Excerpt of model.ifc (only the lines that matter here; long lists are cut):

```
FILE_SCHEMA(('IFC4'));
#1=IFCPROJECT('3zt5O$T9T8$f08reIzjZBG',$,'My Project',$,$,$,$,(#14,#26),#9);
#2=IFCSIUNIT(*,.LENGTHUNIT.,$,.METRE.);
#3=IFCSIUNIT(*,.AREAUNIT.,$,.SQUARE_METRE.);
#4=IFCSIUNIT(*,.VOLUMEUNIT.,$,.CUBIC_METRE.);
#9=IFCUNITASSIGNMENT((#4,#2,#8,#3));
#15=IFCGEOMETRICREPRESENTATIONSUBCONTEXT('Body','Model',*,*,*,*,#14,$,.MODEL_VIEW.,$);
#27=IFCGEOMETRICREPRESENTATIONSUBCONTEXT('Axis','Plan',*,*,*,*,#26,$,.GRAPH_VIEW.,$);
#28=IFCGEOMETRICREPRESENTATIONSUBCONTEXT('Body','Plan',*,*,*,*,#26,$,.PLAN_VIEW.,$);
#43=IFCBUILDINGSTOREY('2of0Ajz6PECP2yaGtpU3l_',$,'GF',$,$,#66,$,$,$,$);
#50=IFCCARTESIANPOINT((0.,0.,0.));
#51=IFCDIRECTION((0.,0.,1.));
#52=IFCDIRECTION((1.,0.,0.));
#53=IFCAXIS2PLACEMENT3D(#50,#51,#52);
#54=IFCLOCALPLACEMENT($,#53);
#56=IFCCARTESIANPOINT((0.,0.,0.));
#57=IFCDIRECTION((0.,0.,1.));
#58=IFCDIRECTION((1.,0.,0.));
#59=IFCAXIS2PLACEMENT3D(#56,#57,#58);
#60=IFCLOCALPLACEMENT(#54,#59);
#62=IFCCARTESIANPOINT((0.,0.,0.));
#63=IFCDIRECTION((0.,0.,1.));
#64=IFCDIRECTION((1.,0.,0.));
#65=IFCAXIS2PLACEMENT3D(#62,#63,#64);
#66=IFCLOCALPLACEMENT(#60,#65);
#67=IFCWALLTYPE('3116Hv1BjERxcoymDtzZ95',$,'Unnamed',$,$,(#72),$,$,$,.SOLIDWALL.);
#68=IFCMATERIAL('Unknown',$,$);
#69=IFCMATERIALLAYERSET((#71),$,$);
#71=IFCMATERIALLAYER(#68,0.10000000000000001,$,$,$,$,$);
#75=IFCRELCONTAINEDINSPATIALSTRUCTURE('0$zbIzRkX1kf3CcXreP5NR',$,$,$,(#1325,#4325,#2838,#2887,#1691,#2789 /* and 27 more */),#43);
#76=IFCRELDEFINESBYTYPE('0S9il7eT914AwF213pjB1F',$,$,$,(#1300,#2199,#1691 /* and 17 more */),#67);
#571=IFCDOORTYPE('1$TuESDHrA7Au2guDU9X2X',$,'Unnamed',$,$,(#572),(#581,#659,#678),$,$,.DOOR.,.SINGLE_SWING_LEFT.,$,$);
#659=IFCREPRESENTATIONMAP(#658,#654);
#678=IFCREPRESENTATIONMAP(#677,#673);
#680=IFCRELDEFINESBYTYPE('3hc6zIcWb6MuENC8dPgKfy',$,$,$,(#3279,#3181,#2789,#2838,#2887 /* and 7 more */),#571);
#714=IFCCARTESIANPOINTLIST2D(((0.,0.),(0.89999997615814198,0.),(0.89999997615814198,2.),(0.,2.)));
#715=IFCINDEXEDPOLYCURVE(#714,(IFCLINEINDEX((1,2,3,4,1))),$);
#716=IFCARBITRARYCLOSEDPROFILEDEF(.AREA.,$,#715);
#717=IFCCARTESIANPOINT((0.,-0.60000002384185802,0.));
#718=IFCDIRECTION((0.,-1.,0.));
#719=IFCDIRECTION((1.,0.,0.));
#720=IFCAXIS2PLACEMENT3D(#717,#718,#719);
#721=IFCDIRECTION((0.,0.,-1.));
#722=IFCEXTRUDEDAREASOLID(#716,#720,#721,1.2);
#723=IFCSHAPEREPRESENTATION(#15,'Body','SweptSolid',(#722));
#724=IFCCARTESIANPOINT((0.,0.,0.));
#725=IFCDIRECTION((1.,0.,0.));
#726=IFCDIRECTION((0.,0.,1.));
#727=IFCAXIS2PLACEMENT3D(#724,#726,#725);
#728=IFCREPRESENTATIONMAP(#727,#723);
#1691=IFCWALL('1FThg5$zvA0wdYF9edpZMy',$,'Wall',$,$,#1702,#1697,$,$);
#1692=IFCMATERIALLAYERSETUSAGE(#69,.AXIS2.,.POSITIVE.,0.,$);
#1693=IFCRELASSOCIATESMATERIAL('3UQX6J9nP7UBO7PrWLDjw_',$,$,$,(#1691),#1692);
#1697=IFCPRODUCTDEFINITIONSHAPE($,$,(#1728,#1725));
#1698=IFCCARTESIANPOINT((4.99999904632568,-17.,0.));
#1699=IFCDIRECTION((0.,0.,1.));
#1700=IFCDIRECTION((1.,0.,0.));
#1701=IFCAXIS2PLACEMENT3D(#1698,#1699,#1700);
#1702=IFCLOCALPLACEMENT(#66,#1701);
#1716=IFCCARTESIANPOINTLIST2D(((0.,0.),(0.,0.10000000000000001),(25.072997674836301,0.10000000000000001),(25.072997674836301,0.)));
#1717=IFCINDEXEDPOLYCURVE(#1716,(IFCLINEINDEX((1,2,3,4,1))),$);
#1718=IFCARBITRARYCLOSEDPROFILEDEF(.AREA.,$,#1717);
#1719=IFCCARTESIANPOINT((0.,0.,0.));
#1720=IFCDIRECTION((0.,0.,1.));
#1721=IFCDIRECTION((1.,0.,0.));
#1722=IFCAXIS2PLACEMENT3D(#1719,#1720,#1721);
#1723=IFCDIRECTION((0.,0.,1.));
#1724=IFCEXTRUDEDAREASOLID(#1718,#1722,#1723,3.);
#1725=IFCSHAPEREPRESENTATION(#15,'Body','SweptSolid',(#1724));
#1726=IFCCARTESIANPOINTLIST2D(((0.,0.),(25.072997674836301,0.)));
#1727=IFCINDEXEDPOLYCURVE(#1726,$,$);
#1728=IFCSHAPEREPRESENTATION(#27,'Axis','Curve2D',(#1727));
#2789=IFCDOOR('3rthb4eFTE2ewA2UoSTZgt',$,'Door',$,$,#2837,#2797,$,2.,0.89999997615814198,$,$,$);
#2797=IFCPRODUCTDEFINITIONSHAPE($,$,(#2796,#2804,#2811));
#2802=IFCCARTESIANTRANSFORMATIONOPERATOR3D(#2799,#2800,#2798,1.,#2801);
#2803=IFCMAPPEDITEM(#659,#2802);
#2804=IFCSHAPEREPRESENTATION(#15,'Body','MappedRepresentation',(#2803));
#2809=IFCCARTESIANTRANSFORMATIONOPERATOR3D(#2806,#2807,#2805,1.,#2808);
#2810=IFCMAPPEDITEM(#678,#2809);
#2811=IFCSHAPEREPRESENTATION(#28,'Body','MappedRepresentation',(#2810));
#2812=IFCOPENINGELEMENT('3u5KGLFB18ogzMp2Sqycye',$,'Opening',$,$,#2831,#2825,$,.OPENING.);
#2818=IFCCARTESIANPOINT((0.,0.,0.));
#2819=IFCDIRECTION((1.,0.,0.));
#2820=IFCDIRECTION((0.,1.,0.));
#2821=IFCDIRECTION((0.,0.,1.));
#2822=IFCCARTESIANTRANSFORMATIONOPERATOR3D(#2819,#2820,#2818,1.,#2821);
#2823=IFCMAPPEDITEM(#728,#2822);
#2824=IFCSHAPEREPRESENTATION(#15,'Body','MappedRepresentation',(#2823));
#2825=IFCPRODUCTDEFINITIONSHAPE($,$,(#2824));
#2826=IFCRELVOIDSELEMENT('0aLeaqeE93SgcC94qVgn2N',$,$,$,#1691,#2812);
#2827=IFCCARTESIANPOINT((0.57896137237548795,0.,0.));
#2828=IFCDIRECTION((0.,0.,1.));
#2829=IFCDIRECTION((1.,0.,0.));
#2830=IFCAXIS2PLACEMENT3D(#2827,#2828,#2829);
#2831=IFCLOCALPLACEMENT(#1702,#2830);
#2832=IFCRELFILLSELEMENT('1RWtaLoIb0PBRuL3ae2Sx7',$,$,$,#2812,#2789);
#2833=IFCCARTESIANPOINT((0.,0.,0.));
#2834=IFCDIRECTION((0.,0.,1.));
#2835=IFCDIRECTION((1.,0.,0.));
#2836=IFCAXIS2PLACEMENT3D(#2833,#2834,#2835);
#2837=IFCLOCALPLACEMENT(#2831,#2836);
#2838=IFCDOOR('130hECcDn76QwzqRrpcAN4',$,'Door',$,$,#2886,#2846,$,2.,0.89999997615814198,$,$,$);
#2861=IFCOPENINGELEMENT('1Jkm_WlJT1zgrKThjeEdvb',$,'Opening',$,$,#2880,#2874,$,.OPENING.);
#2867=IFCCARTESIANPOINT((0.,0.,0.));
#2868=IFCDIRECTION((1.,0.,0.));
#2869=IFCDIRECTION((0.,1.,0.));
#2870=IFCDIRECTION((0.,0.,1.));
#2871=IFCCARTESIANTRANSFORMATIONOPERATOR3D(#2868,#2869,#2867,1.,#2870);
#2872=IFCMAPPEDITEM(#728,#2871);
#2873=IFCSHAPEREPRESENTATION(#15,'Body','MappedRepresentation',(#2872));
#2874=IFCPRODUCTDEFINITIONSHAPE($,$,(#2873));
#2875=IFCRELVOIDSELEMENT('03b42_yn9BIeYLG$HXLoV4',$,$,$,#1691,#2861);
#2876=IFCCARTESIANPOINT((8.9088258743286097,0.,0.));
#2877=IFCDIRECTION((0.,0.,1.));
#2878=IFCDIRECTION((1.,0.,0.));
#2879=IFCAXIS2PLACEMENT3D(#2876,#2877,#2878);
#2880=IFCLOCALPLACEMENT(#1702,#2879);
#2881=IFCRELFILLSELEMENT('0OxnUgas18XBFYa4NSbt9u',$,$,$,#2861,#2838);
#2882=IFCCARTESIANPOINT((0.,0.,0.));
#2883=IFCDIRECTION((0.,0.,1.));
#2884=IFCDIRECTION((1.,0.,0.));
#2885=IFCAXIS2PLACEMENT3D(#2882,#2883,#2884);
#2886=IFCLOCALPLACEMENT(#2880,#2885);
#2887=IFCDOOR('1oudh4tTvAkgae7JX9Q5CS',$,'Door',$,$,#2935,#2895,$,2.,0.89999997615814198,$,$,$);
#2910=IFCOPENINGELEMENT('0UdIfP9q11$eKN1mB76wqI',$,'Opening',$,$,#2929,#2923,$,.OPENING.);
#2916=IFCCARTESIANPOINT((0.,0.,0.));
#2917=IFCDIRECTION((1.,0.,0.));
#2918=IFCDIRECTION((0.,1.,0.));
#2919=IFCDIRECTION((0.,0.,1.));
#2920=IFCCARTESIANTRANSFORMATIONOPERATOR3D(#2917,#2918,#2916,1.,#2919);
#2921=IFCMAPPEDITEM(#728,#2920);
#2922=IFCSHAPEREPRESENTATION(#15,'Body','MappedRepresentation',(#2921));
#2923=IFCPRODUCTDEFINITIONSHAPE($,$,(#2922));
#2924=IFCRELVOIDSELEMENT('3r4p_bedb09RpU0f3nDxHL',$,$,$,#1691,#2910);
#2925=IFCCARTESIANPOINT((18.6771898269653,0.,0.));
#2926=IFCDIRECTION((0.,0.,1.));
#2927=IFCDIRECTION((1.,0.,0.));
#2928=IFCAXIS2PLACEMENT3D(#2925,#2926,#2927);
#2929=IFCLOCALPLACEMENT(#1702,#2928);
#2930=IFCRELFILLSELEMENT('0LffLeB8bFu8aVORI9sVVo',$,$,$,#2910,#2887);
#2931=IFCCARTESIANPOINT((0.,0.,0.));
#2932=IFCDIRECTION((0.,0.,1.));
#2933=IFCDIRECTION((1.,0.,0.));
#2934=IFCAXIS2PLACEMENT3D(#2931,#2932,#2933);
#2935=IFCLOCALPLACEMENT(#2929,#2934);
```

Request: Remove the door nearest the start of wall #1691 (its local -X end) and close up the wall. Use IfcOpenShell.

```python
import ifcopenshell
import ifcopenshell.api.feature
import ifcopenshell.api.root
import ifcopenshell.geom
import ifcopenshell.util.shape

model = ifcopenshell.open("model.ifc")
settings = ifcopenshell.geom.settings()


def volume(element):
    """Net volume in cubic metres, openings subtracted."""
    shape = ifcopenshell.geom.create_shape(settings, element)
    return ifcopenshell.util.shape.get_volume(shape.geometry)


door = model.by_id(2789)
opening = door.FillsVoids[0].RelatingOpeningElement
wall = opening.VoidsElements[0].RelatingBuildingElement
before = volume(wall)

ifcopenshell.api.root.remove_product(model, product=door)
ifcopenshell.api.feature.remove_feature(model, feature=opening)

after = volume(wall)

print(f"wall volume {before:.3f} -> {after:.3f} m3")

model.write("model_edited.ifc")
```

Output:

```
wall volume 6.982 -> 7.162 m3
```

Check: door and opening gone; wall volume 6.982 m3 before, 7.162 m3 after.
